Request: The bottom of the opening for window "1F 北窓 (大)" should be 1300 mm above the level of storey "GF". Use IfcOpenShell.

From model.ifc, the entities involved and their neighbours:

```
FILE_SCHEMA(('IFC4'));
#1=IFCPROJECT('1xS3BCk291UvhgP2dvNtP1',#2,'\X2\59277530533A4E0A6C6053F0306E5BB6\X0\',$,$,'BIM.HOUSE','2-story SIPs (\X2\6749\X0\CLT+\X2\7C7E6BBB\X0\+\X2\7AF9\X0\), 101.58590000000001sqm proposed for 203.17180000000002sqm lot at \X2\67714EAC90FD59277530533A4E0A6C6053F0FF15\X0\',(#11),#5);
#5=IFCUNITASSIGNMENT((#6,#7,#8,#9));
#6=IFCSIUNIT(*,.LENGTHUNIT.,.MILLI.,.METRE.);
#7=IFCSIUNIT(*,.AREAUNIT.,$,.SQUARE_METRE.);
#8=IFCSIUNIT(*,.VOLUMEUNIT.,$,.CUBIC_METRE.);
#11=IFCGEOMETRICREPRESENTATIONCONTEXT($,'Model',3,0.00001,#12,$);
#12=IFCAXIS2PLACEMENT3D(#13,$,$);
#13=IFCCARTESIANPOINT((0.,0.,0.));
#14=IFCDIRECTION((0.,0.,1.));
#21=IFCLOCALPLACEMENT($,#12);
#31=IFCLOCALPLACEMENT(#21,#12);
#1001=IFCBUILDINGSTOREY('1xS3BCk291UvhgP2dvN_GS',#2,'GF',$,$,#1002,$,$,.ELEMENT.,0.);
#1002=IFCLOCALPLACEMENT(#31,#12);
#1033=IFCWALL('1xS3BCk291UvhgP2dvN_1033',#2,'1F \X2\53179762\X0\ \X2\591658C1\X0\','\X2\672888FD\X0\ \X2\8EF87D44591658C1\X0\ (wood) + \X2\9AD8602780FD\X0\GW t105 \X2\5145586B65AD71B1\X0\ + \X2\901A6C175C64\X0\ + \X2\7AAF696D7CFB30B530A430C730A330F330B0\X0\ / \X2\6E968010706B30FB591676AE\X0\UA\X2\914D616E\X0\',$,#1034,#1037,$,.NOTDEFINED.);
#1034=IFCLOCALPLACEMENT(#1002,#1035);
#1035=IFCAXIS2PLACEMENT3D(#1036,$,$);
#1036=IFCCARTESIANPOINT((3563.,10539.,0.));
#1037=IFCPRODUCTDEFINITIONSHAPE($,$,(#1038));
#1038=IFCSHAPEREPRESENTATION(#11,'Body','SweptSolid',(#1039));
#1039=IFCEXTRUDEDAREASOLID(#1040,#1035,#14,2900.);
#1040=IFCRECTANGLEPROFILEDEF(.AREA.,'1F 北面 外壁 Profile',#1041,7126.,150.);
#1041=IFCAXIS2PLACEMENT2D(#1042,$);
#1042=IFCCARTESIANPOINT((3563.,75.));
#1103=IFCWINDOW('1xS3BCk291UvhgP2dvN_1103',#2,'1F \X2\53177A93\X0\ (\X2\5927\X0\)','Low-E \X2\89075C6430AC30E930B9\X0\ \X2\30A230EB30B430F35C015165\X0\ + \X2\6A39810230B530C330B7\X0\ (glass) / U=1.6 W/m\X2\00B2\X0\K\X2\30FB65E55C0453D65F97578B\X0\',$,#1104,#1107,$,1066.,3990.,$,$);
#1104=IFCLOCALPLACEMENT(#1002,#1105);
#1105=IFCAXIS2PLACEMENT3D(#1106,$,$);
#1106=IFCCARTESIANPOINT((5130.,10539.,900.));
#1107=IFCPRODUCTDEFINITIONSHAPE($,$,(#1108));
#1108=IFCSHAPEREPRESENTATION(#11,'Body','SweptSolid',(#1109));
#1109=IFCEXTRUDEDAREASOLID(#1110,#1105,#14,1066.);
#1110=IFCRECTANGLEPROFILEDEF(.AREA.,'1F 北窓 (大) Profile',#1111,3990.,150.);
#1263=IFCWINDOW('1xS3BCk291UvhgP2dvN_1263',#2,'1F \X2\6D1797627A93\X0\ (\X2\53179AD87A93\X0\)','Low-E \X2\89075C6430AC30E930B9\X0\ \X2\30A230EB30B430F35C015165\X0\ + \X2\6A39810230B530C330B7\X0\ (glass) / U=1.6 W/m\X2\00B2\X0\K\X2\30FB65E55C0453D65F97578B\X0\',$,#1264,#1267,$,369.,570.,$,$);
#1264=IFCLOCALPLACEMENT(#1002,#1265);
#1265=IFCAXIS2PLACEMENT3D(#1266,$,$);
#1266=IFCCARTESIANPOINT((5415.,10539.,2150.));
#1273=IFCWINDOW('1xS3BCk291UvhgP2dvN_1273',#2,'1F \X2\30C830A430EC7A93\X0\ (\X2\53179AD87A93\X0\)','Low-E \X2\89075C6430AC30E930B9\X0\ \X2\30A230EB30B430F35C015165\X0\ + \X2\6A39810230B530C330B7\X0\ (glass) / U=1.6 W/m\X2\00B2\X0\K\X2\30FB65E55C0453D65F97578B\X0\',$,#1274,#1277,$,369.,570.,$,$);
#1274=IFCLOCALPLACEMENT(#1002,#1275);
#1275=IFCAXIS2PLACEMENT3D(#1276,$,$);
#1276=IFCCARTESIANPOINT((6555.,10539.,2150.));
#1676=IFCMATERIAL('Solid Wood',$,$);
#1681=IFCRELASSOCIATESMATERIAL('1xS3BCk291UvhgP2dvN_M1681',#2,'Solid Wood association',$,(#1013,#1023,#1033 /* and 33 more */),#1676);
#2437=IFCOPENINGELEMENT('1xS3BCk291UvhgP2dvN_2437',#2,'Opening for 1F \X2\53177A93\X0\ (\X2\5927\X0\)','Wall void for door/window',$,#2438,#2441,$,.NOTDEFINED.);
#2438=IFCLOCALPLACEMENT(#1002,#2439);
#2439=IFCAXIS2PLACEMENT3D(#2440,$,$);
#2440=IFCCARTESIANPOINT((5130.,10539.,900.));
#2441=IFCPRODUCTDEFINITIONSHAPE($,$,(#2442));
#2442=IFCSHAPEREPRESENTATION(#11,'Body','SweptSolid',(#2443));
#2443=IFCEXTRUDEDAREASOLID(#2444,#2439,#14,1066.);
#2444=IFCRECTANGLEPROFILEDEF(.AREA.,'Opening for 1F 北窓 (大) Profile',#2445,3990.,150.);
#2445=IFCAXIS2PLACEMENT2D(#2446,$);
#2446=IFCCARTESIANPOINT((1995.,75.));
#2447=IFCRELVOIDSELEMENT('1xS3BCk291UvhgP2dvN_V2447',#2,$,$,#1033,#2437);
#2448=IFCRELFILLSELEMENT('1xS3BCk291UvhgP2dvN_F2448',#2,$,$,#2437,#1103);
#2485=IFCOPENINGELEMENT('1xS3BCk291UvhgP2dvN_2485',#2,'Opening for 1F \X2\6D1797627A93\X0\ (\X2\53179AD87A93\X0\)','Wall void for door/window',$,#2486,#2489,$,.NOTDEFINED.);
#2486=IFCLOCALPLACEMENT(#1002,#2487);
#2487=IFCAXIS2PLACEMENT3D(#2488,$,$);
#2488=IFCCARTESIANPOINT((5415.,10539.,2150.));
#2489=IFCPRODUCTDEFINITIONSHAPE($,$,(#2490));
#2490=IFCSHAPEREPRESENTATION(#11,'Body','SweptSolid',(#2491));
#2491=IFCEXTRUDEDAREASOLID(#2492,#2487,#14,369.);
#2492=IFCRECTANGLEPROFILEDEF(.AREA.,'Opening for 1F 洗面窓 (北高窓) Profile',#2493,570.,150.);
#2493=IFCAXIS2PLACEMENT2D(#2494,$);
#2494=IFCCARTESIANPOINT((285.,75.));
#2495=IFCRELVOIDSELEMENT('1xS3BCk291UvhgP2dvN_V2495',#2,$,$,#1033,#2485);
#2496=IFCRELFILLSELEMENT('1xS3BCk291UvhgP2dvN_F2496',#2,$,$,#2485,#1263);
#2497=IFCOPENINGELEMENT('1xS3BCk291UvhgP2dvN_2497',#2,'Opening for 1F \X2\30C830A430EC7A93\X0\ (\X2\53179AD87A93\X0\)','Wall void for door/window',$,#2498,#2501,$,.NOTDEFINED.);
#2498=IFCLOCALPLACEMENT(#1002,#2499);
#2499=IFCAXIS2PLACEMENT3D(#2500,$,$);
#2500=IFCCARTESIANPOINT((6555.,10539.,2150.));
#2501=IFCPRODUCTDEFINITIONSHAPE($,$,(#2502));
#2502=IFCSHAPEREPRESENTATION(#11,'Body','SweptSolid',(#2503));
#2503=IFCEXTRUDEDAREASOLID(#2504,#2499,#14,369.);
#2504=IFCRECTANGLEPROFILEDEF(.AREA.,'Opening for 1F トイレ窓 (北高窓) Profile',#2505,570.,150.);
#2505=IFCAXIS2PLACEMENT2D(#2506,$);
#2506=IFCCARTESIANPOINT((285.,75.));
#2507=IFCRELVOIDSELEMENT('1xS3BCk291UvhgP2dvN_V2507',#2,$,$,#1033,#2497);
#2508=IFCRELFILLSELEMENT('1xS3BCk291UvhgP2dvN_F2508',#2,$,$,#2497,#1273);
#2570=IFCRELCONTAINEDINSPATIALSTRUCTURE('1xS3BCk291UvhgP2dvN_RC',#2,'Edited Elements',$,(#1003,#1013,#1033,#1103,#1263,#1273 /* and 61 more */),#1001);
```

```python
import numpy as np
import ifcopenshell
import ifcopenshell.api.geometry
import ifcopenshell.geom
import ifcopenshell.util.element
import ifcopenshell.util.placement
import ifcopenshell.util.shape
import ifcopenshell.util.unit

model = ifcopenshell.open("model.ifc")
unit_scale = ifcopenshell.util.unit.calculate_unit_scale(model)

window = model.by_guid("1xS3BCk291UvhgP2dvN_1103")
opening = window.FillsVoids[0].RelatingOpeningElement
storey = ifcopenshell.util.element.get_container(window, ifc_class="IfcBuildingStorey")
level = ifcopenshell.util.placement.get_local_placement(storey.ObjectPlacement)[2, 3]

# The opening's origin need not be at the sill, so measure its lowest point.
shape = ifcopenshell.geom.create_shape(ifcopenshell.geom.settings(), opening)
bottom = ifcopenshell.util.shape.get_shape_bottom_elevation(shape, shape.geometry) / unit_scale
dz = level + 1300.0 - bottom

shift = np.array([0.0, 0.0, dz])
# The window is not placed relative to its opening, so move both.
for product in (opening, window):
    matrix = ifcopenshell.util.placement.get_local_placement(product.ObjectPlacement)
    matrix[:3, 3] += shift
    ifcopenshell.api.geometry.edit_object_placement(model, product=product, matrix=matrix, is_si=False)

print(f"moved by {dz * unit_scale:+.3f} m")

model.write("model-out.ifc")
```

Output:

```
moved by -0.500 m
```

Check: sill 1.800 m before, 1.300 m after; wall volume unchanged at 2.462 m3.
